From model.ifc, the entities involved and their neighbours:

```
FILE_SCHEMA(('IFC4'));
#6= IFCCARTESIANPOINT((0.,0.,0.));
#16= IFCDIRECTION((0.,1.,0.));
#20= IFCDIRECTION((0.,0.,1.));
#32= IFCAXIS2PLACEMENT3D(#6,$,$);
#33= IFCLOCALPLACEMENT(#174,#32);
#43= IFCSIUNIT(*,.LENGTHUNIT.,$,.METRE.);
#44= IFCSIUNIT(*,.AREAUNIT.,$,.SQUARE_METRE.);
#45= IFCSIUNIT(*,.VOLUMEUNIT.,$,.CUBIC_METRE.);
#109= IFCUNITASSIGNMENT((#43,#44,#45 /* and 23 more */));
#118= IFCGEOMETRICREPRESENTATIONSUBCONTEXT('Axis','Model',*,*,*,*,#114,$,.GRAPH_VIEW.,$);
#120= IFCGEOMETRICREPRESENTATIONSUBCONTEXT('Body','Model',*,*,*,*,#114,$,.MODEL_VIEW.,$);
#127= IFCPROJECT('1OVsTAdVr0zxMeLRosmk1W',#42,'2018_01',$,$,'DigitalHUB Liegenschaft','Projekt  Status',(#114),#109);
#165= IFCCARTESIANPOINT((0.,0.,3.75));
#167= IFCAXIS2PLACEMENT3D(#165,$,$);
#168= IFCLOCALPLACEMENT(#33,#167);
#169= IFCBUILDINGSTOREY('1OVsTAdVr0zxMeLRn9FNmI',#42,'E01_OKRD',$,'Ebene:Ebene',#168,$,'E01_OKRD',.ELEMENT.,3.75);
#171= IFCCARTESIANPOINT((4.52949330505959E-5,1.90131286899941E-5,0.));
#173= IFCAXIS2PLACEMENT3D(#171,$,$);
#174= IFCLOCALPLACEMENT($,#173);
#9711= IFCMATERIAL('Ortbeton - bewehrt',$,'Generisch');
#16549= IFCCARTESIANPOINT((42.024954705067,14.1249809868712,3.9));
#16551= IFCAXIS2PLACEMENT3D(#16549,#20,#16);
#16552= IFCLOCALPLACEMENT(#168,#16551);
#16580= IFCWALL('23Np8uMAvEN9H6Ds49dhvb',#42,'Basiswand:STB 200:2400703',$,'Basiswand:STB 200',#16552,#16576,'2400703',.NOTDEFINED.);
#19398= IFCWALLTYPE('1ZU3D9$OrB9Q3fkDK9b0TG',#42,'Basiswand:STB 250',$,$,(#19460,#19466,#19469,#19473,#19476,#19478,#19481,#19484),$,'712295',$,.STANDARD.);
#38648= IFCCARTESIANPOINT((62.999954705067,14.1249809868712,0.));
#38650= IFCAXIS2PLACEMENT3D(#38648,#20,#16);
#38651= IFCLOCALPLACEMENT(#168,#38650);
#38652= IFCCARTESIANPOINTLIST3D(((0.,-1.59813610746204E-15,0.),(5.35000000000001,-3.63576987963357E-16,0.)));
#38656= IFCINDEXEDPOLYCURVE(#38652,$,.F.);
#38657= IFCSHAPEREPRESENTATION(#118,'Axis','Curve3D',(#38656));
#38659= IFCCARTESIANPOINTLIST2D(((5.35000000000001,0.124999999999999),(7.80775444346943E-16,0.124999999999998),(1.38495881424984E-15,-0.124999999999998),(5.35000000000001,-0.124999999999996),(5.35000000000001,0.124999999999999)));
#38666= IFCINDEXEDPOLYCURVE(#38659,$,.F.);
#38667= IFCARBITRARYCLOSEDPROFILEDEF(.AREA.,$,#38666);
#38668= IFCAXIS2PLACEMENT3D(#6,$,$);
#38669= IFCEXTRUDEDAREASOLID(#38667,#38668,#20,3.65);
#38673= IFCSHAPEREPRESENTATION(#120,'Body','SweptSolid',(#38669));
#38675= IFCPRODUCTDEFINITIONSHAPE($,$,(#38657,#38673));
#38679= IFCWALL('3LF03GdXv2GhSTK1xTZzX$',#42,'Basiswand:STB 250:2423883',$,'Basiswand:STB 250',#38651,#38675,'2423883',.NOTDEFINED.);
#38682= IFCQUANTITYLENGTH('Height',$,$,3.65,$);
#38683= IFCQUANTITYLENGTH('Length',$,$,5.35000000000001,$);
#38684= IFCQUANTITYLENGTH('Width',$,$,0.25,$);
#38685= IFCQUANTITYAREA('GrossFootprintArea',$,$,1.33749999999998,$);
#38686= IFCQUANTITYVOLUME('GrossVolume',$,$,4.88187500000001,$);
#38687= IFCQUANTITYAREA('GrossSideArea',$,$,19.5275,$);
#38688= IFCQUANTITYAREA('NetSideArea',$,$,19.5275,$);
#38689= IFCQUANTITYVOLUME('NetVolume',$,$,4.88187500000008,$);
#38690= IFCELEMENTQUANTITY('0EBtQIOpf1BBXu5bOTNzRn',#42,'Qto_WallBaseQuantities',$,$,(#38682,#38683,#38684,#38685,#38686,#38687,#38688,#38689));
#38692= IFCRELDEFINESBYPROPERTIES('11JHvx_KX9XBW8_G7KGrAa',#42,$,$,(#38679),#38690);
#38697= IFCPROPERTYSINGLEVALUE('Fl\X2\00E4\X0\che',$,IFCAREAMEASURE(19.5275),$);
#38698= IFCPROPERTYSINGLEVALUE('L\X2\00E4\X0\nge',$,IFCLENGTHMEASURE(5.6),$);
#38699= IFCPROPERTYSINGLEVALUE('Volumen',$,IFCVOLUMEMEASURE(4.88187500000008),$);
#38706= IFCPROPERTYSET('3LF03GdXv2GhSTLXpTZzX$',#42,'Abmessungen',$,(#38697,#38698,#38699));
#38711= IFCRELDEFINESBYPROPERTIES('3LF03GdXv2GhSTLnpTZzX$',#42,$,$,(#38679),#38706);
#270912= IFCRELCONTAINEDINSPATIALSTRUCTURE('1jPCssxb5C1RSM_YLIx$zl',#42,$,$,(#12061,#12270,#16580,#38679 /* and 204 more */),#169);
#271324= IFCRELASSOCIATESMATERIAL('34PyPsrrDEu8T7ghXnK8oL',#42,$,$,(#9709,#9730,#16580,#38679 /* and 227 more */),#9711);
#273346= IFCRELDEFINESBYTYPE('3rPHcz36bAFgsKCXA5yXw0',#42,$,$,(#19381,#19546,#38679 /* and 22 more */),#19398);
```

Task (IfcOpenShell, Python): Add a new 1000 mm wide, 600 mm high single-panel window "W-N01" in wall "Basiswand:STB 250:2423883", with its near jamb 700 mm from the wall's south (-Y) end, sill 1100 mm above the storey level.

```python
import numpy as np
import ifcopenshell
import ifcopenshell.api.feature
import ifcopenshell.api.geometry
import ifcopenshell.api.pset
import ifcopenshell.api.root
import ifcopenshell.api.spatial
import ifcopenshell.geom
import ifcopenshell.util.element
import ifcopenshell.util.placement
import ifcopenshell.util.representation
import ifcopenshell.util.shape
import ifcopenshell.util.unit

model = ifcopenshell.open("model.ifc")
unit_scale = ifcopenshell.util.unit.calculate_unit_scale(model)
area_scale = ifcopenshell.util.unit.calculate_unit_scale(model, "AREAUNIT")
volume_scale = ifcopenshell.util.unit.calculate_unit_scale(model, "VOLUMEUNIT")
settings = ifcopenshell.geom.settings()


def volume(element):
    """Net volume in cubic metres, openings subtracted."""
    shape = ifcopenshell.geom.create_shape(settings, element)
    return ifcopenshell.util.shape.get_volume(shape.geometry)


wall = model.by_guid("3LF03GdXv2GhSTK1xTZzX$")
storey = ifcopenshell.util.element.get_container(wall, ifc_class="IfcBuildingStorey")
context = ifcopenshell.util.representation.get_context(model, "Model", "Body", "MODEL_VIEW")
before = volume(wall)

width, height, from_end, sill = 1, 0.6, 0.7, 1.1  # metres

# The wall runs along its own X axis, and the end named is its -X end.
wall_shape = ifcopenshell.geom.create_shape(settings, wall)
x, y, z = ifcopenshell.util.shape.get_vertices(wall_shape.geometry).T
start = x.min() + from_end
face, thickness = float(y.min()), float(y.max() - y.min())
wall_matrix = ifcopenshell.util.placement.get_local_placement(wall.ObjectPlacement)
level = ifcopenshell.util.placement.get_local_placement(storey.ObjectPlacement)[2, 3]


def in_wall(x, y):
    """Placement at x, y metres in the wall's axes, at sill height."""
    matrix = wall_matrix.copy()
    matrix[:, 3] = wall_matrix @ np.array([x / unit_scale, y / unit_scale, 0.0, 1.0])
    matrix[2, 3] = level + sill / unit_scale
    return matrix


# Opening: a box that overshoots both wall faces by 50 mm.
opening = ifcopenshell.api.root.create_entity(model, ifc_class="IfcOpeningElement", predefined_type="OPENING")
box = ifcopenshell.api.geometry.add_wall_representation(
    model, context=context, length=width, height=height, thickness=thickness + 0.1
)
ifcopenshell.api.geometry.assign_representation(model, product=opening, representation=box)
ifcopenshell.api.geometry.edit_object_placement(model, product=opening, matrix=in_wall(start, face - 0.05), is_si=False)
ifcopenshell.api.feature.add_feature(model, feature=opening, element=wall)

window = ifcopenshell.api.root.create_entity(model, ifc_class="IfcWindow", name="W-N01", predefined_type="WINDOW")
window.OverallWidth, window.OverallHeight = width / unit_scale, height / unit_scale
window.PartitioningType = "SINGLE_PANEL"
body = ifcopenshell.api.geometry.add_window_representation(
    model,
    context=context,
    overall_width=window.OverallWidth,
    overall_height=window.OverallHeight,
    partition_type="SINGLE_PANEL",
)
ifcopenshell.api.geometry.assign_representation(model, product=window, representation=body)
ifcopenshell.api.spatial.assign_container(model, products=[window], relating_structure=storey)
ifcopenshell.api.feature.add_filling(model, opening=opening, element=window)

# Centre the window in the wall's thickness.
ifcopenshell.api.geometry.edit_object_placement(model, product=window, matrix=in_wall(start, face), is_si=False)
window_shape = ifcopenshell.geom.create_shape(settings, window)
depth = ifcopenshell.util.shape.get_vertices(window_shape.geometry)[:, 1]
offset = face + thickness / 2 - (depth.min() + depth.max()) / 2
ifcopenshell.api.geometry.edit_object_placement(model, product=window, matrix=in_wall(start, offset), is_si=False)

after = volume(wall)

# Update the wall's stored quantities.
qto = model.by_id(ifcopenshell.util.element.get_pset(wall, "Qto_WallBaseQuantities", should_inherit=False)["id"])
ifcopenshell.api.pset.edit_qto(model, qto=qto, properties={
    "NetSideArea": after / thickness / area_scale,
    "NetVolume": after / volume_scale,
})
pset = model.by_id(ifcopenshell.util.element.get_pset(wall, "Abmessungen", should_inherit=False)["id"])
ifcopenshell.api.pset.edit_pset(model, pset=pset, properties={
    "Fläche": model.create_entity("IfcAreaMeasure", after / thickness / area_scale),
    "Volumen": model.create_entity("IfcVolumeMeasure", after / volume_scale),
})

print(f"wall volume {before:.3f} -> {after:.3f} m3")

model.write("model_v2.ifc")
```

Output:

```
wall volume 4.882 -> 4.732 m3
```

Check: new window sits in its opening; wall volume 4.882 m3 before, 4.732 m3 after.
